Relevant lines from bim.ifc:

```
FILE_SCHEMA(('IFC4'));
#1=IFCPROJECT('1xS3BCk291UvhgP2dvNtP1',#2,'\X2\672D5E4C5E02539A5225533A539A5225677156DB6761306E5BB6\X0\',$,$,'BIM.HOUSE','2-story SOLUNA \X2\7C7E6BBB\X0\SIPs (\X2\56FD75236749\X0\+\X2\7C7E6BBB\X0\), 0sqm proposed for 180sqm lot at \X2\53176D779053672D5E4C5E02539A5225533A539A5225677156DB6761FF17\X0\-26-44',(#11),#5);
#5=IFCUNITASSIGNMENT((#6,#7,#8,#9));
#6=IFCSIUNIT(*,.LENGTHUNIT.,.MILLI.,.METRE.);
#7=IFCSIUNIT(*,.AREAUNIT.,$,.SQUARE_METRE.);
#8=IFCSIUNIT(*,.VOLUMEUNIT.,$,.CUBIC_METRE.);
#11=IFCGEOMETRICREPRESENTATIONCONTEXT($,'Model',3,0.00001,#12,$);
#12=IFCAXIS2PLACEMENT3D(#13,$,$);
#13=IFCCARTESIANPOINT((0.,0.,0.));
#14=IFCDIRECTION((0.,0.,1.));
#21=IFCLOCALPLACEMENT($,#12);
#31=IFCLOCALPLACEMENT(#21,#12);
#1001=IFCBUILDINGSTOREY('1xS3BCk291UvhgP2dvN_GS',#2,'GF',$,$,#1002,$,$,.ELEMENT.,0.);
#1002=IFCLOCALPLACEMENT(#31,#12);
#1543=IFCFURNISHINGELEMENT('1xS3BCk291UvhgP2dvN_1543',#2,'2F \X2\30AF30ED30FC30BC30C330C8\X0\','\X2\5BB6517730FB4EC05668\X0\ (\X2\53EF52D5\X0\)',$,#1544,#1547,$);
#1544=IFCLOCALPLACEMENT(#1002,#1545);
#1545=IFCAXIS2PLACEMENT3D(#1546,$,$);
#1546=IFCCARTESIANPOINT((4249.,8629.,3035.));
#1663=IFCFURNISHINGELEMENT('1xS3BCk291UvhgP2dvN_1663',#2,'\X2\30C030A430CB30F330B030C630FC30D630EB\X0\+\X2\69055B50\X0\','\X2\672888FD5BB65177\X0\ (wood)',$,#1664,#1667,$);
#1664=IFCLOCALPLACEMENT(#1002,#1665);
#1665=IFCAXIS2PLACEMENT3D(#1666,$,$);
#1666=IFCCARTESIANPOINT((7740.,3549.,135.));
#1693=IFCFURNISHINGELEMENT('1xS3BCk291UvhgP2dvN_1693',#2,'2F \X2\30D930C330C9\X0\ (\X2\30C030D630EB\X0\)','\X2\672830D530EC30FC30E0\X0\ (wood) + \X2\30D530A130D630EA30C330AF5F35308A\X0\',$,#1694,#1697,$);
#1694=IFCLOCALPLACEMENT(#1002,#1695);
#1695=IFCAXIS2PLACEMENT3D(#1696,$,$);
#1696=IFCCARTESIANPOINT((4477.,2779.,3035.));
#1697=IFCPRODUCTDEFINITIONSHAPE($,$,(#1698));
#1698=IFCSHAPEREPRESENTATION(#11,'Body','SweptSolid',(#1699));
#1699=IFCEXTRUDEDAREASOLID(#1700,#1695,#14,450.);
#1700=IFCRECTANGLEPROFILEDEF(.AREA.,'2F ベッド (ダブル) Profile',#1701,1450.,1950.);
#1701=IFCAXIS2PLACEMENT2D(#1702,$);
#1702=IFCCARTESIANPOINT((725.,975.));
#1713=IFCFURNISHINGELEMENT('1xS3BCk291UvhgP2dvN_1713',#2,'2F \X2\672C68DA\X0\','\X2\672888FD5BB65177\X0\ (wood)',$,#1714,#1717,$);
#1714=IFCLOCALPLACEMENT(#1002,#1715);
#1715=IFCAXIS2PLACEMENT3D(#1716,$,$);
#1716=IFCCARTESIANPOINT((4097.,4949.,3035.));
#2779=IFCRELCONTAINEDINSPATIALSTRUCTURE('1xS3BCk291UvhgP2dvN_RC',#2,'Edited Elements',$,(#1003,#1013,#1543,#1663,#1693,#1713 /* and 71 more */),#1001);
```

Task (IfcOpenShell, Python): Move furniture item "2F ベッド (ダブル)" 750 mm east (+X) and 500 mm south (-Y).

```python
import ifcopenshell
import ifcopenshell.api.geometry
import ifcopenshell.util.placement

model = ifcopenshell.open("bim.ifc")

item = model.by_id(1693)
matrix = ifcopenshell.util.placement.get_local_placement(item.ObjectPlacement)
matrix[0, 3] += 750.0
matrix[1, 3] -= 500.0
ifcopenshell.api.geometry.edit_object_placement(model, product=item, matrix=matrix, is_si=False)

print(ifcopenshell.util.placement.get_local_placement(item.ObjectPlacement).round(3) + 0.0)

model.write("bim_edited.ifc")
```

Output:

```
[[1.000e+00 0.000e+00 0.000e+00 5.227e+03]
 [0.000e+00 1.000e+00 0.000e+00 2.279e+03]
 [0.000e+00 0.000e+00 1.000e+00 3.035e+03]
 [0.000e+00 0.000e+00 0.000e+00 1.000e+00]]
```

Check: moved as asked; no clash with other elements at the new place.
